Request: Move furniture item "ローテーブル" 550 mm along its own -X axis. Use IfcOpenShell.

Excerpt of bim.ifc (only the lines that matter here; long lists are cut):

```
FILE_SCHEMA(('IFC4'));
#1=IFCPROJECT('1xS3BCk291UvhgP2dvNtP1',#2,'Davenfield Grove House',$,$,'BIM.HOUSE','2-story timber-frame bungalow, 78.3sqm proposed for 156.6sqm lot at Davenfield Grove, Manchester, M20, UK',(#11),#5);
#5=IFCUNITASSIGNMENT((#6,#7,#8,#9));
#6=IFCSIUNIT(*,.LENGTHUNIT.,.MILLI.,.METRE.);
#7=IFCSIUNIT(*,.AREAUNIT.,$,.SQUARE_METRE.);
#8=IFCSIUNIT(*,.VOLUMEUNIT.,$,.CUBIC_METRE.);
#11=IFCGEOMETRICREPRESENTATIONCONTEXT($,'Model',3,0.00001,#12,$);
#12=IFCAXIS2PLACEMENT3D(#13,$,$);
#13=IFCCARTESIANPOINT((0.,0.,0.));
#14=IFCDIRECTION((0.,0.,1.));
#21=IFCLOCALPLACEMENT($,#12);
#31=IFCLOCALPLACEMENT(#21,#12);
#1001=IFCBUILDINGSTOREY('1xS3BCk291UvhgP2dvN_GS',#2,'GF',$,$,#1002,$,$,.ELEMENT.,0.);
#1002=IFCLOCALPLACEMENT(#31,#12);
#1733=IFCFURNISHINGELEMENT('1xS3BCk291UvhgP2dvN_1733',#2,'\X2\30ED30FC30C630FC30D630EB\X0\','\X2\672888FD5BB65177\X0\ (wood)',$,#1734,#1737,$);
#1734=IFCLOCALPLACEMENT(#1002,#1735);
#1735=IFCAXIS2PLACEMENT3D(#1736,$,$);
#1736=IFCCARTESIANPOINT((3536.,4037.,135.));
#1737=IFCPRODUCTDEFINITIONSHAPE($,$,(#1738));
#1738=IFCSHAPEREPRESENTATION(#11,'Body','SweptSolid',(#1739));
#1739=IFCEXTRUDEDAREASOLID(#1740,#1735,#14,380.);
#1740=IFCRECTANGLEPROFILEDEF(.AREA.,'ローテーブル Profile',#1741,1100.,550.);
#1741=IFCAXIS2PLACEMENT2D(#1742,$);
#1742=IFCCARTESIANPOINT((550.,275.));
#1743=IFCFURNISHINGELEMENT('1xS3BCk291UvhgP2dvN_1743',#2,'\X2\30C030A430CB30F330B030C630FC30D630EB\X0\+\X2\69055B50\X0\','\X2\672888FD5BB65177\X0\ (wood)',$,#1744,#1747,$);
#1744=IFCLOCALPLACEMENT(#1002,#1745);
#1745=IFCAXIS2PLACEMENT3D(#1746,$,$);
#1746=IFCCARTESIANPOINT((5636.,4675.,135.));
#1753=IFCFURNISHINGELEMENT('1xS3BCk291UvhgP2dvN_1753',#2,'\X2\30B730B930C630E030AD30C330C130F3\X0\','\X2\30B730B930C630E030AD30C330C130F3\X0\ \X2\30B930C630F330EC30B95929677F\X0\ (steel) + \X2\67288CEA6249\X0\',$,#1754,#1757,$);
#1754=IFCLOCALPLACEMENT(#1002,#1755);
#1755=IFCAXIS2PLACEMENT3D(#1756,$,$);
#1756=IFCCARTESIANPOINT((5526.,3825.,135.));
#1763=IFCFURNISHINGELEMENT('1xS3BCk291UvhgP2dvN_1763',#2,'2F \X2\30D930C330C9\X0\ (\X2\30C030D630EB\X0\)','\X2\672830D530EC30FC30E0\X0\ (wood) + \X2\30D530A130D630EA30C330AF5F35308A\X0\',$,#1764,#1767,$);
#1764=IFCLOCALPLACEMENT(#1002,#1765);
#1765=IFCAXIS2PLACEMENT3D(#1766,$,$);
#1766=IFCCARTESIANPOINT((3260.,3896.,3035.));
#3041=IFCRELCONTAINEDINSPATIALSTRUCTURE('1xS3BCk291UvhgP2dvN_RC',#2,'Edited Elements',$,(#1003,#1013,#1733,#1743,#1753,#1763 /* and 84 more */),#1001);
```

```python
import ifcopenshell
import ifcopenshell.api.geometry
import ifcopenshell.util.placement
import ifcopenshell.util.unit

model = ifcopenshell.open("bim.ifc")
unit_scale = ifcopenshell.util.unit.calculate_unit_scale(model)

item = model.by_guid("1xS3BCk291UvhgP2dvN_1733")
matrix = ifcopenshell.util.placement.get_local_placement(item.ObjectPlacement)
matrix[:3, 3] -= matrix[:3, 0] * 0.55 / unit_scale
ifcopenshell.api.geometry.edit_object_placement(model, product=item, matrix=matrix, is_si=False)

print(ifcopenshell.util.placement.get_local_placement(item.ObjectPlacement).round(3) + 0.0)

model.write("bim_rev.ifc")
```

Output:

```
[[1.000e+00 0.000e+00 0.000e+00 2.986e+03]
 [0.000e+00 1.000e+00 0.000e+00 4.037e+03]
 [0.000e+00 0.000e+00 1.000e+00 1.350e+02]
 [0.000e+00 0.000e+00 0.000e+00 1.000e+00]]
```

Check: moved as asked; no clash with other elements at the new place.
